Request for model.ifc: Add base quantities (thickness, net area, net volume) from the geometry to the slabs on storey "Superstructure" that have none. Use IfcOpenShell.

First a look at what the model holds.

```python
import ifcopenshell
import ifcopenshell.util.element
import ifcopenshell.util.unit

model = ifcopenshell.open("model.ifc")
print(model.schema)
for unit_type in ("LENGTHUNIT", "AREAUNIT", "VOLUMEUNIT"):
    print(unit_type, ifcopenshell.util.unit.calculate_unit_scale(model, unit_type))
storey = next(s for s in model.by_type("IfcBuildingStorey") if s.Name == "Superstructure")
slabs = [e for e in ifcopenshell.util.element.get_decomposition(storey) if e.is_a("IfcSlab")]
for e in sorted(slabs, key=lambda e: e.id()):
    print(e.id(), e.is_a(), e.Name, list(ifcopenshell.util.element.get_psets(e, qtos_only=True)), sep=" | ")
```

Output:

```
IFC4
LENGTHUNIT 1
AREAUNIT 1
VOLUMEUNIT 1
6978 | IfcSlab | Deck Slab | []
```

```python
import ifcopenshell
import ifcopenshell.api.pset
import ifcopenshell.geom
import ifcopenshell.util.element
import ifcopenshell.util.shape
import ifcopenshell.util.unit

model = ifcopenshell.open("model.ifc")
unit_scale = ifcopenshell.util.unit.calculate_unit_scale(model)
area_scale = ifcopenshell.util.unit.calculate_unit_scale(model, "AREAUNIT")
volume_scale = ifcopenshell.util.unit.calculate_unit_scale(model, "VOLUMEUNIT")
settings = ifcopenshell.geom.settings()

storey = next(s for s in model.by_type("IfcBuildingStorey") if s.Name == "Superstructure")
slabs = [e for e in ifcopenshell.util.element.get_decomposition(storey) if e.is_a("IfcSlab")]

for e in sorted(slabs, key=lambda e: e.id()):
    if ifcopenshell.util.element.get_psets(e, qtos_only=True, should_inherit=False):
        continue
    # Geometry comes back in metres, in the element's own axes.
    shape = ifcopenshell.geom.create_shape(settings, e)
    values = {
        "Width": ifcopenshell.util.shape.get_z(shape.geometry) / unit_scale,
        "NetArea": ifcopenshell.util.shape.get_footprint_area(shape.geometry) / area_scale,
        "NetVolume": ifcopenshell.util.shape.get_volume(shape.geometry) / volume_scale,
    }
    qto = ifcopenshell.api.pset.add_qto(model, product=e, name="Qto_SlabBaseQuantities")
    ifcopenshell.api.pset.edit_qto(model, qto=qto, properties=values)
    print(e.id(), {k: round(v, 3) for k, v in values.items()})

model.write("model_edited.ifc")
```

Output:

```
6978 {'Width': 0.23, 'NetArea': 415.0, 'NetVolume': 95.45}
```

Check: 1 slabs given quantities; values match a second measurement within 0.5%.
